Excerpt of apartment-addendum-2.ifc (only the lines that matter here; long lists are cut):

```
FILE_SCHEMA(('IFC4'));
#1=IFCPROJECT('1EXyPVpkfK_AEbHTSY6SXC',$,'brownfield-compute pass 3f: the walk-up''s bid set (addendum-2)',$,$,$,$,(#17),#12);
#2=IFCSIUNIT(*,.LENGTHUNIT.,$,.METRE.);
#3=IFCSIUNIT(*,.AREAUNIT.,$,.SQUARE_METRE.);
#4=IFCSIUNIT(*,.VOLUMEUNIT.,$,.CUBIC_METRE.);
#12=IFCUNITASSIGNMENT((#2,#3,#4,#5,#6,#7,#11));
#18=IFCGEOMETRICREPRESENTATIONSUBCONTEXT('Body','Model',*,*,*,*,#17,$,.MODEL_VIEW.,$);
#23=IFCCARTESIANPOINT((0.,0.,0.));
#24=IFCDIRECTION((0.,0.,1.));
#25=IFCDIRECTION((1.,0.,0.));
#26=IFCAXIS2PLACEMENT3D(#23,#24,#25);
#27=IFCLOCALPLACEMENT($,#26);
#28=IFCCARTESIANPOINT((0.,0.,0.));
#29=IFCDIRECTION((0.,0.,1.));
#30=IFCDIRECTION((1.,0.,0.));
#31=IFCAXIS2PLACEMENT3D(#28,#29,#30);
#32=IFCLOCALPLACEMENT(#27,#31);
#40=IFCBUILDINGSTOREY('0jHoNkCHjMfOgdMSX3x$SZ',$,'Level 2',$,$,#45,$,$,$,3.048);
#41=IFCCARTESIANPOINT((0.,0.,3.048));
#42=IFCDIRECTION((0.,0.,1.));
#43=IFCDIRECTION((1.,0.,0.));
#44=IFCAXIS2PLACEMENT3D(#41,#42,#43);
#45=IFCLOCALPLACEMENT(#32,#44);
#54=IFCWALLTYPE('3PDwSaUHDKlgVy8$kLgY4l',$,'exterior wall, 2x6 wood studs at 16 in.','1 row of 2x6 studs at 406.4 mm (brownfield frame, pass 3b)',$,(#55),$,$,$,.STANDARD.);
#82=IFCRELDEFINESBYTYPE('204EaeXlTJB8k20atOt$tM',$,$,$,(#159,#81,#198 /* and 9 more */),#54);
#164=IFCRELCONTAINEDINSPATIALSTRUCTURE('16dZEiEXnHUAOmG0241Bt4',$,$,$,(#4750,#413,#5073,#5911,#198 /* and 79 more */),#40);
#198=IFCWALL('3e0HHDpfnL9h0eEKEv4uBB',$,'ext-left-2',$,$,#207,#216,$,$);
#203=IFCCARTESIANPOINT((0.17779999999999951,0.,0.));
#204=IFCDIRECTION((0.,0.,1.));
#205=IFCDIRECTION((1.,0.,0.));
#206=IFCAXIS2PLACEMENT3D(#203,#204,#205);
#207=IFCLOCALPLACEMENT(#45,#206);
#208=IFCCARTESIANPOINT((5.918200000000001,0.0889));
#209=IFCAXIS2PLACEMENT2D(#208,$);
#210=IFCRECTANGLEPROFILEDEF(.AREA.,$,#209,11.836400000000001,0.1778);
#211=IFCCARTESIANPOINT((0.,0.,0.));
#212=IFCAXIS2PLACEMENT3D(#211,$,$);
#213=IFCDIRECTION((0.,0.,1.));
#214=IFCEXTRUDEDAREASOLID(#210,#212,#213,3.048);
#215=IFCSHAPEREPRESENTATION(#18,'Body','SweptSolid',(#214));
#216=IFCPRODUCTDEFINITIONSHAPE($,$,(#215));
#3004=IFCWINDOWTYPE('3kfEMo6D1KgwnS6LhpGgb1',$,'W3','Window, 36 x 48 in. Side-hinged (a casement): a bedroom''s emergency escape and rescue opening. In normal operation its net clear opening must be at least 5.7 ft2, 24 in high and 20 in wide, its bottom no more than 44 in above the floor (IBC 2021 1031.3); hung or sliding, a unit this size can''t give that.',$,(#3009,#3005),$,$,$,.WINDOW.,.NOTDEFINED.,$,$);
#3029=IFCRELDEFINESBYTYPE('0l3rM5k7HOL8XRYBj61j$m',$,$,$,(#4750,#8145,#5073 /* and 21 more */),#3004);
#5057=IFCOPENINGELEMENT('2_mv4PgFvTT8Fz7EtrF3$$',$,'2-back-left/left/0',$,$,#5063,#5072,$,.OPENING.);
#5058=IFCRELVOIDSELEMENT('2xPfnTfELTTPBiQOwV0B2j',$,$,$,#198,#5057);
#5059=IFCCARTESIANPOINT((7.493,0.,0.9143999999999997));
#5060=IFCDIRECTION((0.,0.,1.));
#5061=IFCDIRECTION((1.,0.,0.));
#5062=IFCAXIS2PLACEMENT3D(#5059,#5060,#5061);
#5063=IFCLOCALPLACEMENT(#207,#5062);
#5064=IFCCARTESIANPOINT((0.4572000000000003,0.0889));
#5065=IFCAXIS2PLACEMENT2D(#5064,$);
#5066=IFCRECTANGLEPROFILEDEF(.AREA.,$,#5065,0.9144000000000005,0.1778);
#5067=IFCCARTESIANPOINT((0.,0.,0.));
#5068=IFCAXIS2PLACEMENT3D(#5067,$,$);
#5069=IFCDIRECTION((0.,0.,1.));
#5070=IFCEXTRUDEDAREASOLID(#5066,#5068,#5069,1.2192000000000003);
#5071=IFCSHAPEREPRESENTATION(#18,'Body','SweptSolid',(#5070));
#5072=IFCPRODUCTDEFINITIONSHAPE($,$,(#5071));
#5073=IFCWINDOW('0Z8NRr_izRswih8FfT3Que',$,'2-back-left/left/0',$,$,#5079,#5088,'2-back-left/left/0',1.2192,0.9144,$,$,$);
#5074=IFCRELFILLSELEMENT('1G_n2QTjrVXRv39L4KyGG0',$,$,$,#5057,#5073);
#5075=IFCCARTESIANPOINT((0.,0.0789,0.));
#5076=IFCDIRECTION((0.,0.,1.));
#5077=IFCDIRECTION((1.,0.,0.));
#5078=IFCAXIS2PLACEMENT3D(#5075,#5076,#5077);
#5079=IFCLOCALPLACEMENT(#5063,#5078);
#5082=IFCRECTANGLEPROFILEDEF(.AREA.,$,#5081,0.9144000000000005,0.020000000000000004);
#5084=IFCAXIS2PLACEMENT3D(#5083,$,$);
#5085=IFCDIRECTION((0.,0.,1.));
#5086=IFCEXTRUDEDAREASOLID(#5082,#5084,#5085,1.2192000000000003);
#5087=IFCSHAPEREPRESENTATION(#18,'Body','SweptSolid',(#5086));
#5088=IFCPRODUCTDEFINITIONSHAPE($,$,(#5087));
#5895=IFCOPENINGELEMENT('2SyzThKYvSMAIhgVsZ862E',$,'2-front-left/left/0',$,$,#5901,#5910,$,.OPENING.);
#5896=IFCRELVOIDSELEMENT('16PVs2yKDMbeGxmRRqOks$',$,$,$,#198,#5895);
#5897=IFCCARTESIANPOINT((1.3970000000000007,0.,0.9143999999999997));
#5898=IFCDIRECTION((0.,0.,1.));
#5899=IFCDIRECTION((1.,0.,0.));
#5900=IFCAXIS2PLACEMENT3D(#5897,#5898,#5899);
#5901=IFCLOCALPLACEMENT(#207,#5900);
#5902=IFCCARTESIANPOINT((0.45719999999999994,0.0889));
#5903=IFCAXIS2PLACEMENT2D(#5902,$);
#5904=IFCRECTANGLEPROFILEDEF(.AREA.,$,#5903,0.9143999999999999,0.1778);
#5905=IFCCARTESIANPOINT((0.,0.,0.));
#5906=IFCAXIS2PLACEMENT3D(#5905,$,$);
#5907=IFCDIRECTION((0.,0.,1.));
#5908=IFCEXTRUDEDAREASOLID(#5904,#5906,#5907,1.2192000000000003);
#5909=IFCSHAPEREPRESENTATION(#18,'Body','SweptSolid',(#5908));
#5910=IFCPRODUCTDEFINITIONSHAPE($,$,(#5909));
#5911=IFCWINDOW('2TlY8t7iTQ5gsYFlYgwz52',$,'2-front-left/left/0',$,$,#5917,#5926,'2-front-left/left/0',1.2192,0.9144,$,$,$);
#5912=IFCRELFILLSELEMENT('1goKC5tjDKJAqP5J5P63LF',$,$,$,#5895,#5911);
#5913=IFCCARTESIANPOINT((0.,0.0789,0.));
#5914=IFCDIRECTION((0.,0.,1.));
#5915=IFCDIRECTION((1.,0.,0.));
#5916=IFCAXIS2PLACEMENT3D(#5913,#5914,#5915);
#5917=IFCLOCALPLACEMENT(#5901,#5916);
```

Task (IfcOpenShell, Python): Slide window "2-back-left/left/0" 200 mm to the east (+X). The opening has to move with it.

```python
import ifcopenshell
import ifcopenshell.api.geometry
import ifcopenshell.util.placement
import ifcopenshell.util.unit

model = ifcopenshell.open("apartment-addendum-2.ifc")
unit_scale = ifcopenshell.util.unit.calculate_unit_scale(model)

window = model.by_guid("0Z8NRr_izRswih8FfT3Que")
opening = window.FillsVoids[0].RelatingOpeningElement
wall = opening.VoidsElements[0].RelatingBuildingElement

wall_matrix = ifcopenshell.util.placement.get_local_placement(wall.ObjectPlacement)
shift = wall_matrix[:3, 0] * 0.2 / unit_scale
before = ifcopenshell.util.placement.get_local_placement(window.ObjectPlacement)[:3, 3].copy()

# The window is placed relative to its opening, so it follows when the opening moves.
matrix = ifcopenshell.util.placement.get_local_placement(opening.ObjectPlacement)
matrix[:3, 3] += shift
ifcopenshell.api.geometry.edit_object_placement(
    model, product=opening, matrix=matrix, is_si=False, should_transform_children=True
)

after = ifcopenshell.util.placement.get_local_placement(window.ObjectPlacement)[:3, 3]
print("window moved by", (after - before).round(3) + 0.0)

model.write("apartment-addendum-2_edited.ifc")
```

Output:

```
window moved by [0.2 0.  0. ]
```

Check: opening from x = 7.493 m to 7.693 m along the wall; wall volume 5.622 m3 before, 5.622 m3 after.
